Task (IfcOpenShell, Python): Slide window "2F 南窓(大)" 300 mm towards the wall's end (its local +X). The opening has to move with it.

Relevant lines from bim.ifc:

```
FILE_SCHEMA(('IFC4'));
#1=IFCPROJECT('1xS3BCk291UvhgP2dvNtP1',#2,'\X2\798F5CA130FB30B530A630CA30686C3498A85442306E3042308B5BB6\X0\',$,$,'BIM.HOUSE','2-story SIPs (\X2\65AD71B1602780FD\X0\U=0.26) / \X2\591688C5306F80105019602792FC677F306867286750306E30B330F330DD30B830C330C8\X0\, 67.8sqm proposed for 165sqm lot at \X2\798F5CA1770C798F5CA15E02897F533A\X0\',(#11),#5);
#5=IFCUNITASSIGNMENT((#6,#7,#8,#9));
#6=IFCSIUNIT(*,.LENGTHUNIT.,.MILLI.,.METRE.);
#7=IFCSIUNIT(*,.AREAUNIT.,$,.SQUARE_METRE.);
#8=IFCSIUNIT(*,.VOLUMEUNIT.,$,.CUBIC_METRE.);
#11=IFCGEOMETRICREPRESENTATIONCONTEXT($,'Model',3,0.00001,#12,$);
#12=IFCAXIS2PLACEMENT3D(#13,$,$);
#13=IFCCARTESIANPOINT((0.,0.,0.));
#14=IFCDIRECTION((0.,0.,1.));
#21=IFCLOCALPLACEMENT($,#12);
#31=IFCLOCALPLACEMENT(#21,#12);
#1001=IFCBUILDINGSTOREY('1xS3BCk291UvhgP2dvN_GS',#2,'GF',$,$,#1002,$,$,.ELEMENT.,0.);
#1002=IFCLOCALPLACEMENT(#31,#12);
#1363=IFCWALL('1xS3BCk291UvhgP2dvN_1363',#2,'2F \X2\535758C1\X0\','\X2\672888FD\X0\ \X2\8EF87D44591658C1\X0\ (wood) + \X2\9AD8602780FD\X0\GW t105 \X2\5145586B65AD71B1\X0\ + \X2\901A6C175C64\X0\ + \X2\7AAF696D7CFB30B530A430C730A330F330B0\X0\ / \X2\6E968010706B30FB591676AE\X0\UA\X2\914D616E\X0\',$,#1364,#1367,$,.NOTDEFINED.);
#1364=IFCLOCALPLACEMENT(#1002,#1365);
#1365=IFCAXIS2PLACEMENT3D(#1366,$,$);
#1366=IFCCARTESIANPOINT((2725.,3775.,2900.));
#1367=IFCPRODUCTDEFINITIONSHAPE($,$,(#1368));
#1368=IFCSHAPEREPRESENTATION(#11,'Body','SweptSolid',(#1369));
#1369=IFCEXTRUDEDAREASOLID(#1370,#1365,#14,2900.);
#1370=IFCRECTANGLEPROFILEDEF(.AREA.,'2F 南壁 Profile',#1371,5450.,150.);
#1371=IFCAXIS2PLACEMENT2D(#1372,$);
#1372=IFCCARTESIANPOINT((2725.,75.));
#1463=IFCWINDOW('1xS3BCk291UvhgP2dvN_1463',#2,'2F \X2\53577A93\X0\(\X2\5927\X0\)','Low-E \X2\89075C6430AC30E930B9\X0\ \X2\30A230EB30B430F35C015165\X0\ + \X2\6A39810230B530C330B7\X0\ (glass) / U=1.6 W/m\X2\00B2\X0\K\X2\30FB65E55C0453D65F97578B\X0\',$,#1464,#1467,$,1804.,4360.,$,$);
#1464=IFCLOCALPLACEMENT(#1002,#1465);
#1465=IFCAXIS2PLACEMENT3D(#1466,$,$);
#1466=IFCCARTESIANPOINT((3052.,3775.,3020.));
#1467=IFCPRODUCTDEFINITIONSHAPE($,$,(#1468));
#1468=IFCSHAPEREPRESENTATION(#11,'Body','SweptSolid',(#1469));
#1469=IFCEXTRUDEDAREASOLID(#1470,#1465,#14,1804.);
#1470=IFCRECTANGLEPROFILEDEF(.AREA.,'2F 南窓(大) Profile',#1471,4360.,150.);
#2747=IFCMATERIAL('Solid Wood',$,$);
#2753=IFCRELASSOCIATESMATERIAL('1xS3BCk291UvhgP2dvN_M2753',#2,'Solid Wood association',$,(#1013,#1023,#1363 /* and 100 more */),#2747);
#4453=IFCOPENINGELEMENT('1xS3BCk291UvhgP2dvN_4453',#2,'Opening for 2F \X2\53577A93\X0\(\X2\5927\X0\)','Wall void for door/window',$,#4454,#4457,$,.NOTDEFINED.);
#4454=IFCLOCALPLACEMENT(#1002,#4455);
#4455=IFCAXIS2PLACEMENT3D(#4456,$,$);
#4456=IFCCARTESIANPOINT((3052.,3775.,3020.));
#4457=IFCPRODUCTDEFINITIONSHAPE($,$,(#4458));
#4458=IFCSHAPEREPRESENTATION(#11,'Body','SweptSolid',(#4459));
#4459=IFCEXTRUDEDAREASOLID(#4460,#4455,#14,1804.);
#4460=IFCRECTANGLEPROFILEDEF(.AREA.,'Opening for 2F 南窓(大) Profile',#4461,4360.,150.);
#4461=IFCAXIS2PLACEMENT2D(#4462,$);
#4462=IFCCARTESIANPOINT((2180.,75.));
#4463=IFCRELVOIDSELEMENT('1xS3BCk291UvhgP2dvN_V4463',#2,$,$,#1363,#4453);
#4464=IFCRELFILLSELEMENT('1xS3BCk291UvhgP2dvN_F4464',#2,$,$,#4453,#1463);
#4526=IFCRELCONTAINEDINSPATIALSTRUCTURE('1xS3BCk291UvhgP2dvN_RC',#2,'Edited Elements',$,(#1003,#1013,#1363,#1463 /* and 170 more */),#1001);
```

```python
import ifcopenshell
import ifcopenshell.api.geometry
import ifcopenshell.util.placement
import ifcopenshell.util.unit

model = ifcopenshell.open("bim.ifc")
unit_scale = ifcopenshell.util.unit.calculate_unit_scale(model)

window = model.by_guid("1xS3BCk291UvhgP2dvN_1463")
opening = window.FillsVoids[0].RelatingOpeningElement
wall = opening.VoidsElements[0].RelatingBuildingElement

wall_matrix = ifcopenshell.util.placement.get_local_placement(wall.ObjectPlacement)
shift = wall_matrix[:3, 0] * 0.3 / unit_scale
before = ifcopenshell.util.placement.get_local_placement(window.ObjectPlacement)[:3, 3].copy()

# The window is not placed relative to its opening, so move both.
for product in (opening, window):
    matrix = ifcopenshell.util.placement.get_local_placement(product.ObjectPlacement)
    matrix[:3, 3] += shift
    ifcopenshell.api.geometry.edit_object_placement(model, product=product, matrix=matrix, is_si=False)

after = ifcopenshell.util.placement.get_local_placement(window.ObjectPlacement)[:3, 3]
print("window moved by", (after - before).round(3) + 0.0)

model.write("bim_v2.ifc")
```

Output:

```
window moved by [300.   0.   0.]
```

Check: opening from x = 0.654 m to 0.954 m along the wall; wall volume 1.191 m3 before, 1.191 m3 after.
